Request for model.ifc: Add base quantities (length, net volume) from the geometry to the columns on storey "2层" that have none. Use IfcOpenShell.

First a look at what the model holds.

```python
import ifcopenshell
import ifcopenshell.util.element
import ifcopenshell.util.unit

model = ifcopenshell.open("model.ifc")
print(model.schema)
for unit_type in ("LENGTHUNIT", "AREAUNIT", "VOLUMEUNIT"):
    print(unit_type, ifcopenshell.util.unit.calculate_unit_scale(model, unit_type))
storey = next(s for s in model.by_type("IfcBuildingStorey") if s.Name == "2层")
columns = [e for e in ifcopenshell.util.element.get_decomposition(storey) if e.is_a("IfcColumn")]
for e in sorted(columns, key=lambda e: e.id()):
    print(e.id(), e.is_a(), e.Name, list(ifcopenshell.util.element.get_psets(e, qtos_only=True)), sep=" | ")
```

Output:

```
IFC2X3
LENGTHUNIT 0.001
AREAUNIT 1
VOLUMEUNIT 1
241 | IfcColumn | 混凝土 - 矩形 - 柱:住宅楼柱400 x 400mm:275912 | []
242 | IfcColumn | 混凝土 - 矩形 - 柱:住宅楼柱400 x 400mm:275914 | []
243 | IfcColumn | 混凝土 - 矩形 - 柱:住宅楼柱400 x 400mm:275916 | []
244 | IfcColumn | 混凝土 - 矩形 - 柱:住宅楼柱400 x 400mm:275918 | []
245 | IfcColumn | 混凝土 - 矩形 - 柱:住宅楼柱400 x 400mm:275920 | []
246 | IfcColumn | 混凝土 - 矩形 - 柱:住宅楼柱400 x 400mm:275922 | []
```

```python
import ifcopenshell
import ifcopenshell.api.pset
import ifcopenshell.geom
import ifcopenshell.util.element
import ifcopenshell.util.shape
import ifcopenshell.util.unit

model = ifcopenshell.open("model.ifc")
unit_scale = ifcopenshell.util.unit.calculate_unit_scale(model)
volume_scale = ifcopenshell.util.unit.calculate_unit_scale(model, "VOLUMEUNIT")
settings = ifcopenshell.geom.settings()

storey = next(s for s in model.by_type("IfcBuildingStorey") if s.Name == "2层")
columns = [e for e in ifcopenshell.util.element.get_decomposition(storey) if e.is_a("IfcColumn")]

for e in sorted(columns, key=lambda e: e.id()):
    if ifcopenshell.util.element.get_psets(e, qtos_only=True, should_inherit=False):
        continue
    # Geometry comes back in metres, in the element's own axes.
    shape = ifcopenshell.geom.create_shape(settings, e)
    values = {
        "Length": ifcopenshell.util.shape.get_z(shape.geometry) / unit_scale,
        "NetVolume": ifcopenshell.util.shape.get_volume(shape.geometry) / volume_scale,
    }
    qto = ifcopenshell.api.pset.add_qto(model, product=e, name="BaseQuantities")
    ifcopenshell.api.pset.edit_qto(model, qto=qto, properties=values)
    print(e.id(), {k: round(v, 3) for k, v in values.items()})

model.write("model-out.ifc")
```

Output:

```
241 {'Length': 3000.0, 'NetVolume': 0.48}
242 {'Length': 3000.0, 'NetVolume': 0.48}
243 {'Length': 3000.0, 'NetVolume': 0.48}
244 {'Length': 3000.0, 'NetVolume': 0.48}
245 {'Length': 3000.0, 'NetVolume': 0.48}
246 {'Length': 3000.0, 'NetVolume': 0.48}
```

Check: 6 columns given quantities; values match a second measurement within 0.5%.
